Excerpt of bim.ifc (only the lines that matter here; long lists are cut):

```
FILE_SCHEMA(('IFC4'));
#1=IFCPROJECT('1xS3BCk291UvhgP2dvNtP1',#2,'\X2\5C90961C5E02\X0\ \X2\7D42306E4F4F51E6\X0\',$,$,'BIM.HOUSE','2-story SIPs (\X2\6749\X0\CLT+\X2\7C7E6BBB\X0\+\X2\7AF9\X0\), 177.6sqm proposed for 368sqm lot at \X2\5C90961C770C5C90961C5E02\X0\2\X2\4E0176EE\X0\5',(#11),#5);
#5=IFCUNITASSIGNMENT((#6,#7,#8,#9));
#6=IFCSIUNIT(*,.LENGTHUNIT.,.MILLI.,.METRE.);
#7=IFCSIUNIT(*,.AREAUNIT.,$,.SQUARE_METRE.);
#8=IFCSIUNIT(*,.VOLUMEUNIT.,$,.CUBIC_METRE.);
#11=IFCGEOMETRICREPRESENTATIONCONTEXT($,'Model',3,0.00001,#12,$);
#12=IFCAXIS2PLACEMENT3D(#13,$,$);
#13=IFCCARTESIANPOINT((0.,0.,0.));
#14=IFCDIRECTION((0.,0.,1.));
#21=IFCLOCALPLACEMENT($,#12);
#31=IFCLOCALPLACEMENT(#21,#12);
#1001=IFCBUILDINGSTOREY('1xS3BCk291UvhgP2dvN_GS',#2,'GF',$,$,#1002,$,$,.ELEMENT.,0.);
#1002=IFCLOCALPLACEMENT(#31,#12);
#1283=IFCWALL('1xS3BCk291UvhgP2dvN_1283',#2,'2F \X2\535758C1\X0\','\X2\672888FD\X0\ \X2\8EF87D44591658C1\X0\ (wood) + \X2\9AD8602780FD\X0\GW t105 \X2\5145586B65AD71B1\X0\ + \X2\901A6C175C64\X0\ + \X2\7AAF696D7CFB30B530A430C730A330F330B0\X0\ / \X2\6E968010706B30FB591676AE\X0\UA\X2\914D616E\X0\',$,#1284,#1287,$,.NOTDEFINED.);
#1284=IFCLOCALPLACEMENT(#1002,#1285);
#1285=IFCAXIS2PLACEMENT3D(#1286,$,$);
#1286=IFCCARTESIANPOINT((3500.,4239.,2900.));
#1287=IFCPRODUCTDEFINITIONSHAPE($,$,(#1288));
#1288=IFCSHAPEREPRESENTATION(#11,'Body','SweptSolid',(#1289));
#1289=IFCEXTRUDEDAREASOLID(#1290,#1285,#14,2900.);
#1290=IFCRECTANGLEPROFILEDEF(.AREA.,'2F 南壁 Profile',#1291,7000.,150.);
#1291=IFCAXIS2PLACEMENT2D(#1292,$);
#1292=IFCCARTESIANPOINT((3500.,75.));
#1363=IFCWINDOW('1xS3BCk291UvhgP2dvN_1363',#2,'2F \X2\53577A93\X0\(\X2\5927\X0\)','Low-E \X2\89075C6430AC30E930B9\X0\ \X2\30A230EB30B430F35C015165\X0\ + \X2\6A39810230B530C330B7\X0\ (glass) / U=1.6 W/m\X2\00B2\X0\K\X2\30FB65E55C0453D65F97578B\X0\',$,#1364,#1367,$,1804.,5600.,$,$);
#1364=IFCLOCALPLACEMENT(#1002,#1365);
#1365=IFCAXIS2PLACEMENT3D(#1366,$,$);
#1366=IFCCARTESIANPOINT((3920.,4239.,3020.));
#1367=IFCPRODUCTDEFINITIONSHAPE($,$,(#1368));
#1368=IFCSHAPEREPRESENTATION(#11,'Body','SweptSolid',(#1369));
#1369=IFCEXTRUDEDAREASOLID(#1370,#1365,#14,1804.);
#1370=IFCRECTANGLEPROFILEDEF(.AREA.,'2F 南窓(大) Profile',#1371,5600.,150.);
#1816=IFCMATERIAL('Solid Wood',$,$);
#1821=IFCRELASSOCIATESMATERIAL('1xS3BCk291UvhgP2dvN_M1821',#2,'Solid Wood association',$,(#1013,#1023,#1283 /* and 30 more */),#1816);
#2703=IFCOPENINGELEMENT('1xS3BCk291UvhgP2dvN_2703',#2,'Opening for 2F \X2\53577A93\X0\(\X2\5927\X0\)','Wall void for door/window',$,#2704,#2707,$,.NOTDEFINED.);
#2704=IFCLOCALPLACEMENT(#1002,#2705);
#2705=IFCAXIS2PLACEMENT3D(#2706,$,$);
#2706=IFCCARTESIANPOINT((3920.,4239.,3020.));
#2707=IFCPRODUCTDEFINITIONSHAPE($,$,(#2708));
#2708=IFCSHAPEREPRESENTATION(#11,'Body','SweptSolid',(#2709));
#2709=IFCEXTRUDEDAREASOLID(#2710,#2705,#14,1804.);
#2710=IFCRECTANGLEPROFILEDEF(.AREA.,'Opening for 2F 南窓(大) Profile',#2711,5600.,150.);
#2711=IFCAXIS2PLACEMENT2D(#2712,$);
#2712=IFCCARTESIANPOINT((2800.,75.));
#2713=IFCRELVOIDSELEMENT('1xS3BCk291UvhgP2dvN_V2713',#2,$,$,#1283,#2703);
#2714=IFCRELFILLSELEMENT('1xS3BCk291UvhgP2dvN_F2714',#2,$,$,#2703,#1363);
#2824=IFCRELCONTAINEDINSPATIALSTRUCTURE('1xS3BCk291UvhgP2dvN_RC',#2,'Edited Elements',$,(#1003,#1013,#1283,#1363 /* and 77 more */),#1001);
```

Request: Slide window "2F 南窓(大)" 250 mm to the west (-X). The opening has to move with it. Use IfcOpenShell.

```python
import ifcopenshell
import ifcopenshell.api.geometry
import ifcopenshell.util.placement
import ifcopenshell.util.unit

model = ifcopenshell.open("bim.ifc")
unit_scale = ifcopenshell.util.unit.calculate_unit_scale(model)

window = model.by_id(1363)
opening = window.FillsVoids[0].RelatingOpeningElement
wall = opening.VoidsElements[0].RelatingBuildingElement

wall_matrix = ifcopenshell.util.placement.get_local_placement(wall.ObjectPlacement)
shift = wall_matrix[:3, 0] * -0.25 / unit_scale
before = ifcopenshell.util.placement.get_local_placement(window.ObjectPlacement)[:3, 3].copy()

# The window is not placed relative to its opening, so move both.
for product in (opening, window):
    matrix = ifcopenshell.util.placement.get_local_placement(product.ObjectPlacement)
    matrix[:3, 3] += shift
    ifcopenshell.api.geometry.edit_object_placement(model, product=product, matrix=matrix, is_si=False)

after = ifcopenshell.util.placement.get_local_placement(window.ObjectPlacement)[:3, 3]
print("window moved by", (after - before).round(3) + 0.0)

model.write("bim_edited.ifc")
```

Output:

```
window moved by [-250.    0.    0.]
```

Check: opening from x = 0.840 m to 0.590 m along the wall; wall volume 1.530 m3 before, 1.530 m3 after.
